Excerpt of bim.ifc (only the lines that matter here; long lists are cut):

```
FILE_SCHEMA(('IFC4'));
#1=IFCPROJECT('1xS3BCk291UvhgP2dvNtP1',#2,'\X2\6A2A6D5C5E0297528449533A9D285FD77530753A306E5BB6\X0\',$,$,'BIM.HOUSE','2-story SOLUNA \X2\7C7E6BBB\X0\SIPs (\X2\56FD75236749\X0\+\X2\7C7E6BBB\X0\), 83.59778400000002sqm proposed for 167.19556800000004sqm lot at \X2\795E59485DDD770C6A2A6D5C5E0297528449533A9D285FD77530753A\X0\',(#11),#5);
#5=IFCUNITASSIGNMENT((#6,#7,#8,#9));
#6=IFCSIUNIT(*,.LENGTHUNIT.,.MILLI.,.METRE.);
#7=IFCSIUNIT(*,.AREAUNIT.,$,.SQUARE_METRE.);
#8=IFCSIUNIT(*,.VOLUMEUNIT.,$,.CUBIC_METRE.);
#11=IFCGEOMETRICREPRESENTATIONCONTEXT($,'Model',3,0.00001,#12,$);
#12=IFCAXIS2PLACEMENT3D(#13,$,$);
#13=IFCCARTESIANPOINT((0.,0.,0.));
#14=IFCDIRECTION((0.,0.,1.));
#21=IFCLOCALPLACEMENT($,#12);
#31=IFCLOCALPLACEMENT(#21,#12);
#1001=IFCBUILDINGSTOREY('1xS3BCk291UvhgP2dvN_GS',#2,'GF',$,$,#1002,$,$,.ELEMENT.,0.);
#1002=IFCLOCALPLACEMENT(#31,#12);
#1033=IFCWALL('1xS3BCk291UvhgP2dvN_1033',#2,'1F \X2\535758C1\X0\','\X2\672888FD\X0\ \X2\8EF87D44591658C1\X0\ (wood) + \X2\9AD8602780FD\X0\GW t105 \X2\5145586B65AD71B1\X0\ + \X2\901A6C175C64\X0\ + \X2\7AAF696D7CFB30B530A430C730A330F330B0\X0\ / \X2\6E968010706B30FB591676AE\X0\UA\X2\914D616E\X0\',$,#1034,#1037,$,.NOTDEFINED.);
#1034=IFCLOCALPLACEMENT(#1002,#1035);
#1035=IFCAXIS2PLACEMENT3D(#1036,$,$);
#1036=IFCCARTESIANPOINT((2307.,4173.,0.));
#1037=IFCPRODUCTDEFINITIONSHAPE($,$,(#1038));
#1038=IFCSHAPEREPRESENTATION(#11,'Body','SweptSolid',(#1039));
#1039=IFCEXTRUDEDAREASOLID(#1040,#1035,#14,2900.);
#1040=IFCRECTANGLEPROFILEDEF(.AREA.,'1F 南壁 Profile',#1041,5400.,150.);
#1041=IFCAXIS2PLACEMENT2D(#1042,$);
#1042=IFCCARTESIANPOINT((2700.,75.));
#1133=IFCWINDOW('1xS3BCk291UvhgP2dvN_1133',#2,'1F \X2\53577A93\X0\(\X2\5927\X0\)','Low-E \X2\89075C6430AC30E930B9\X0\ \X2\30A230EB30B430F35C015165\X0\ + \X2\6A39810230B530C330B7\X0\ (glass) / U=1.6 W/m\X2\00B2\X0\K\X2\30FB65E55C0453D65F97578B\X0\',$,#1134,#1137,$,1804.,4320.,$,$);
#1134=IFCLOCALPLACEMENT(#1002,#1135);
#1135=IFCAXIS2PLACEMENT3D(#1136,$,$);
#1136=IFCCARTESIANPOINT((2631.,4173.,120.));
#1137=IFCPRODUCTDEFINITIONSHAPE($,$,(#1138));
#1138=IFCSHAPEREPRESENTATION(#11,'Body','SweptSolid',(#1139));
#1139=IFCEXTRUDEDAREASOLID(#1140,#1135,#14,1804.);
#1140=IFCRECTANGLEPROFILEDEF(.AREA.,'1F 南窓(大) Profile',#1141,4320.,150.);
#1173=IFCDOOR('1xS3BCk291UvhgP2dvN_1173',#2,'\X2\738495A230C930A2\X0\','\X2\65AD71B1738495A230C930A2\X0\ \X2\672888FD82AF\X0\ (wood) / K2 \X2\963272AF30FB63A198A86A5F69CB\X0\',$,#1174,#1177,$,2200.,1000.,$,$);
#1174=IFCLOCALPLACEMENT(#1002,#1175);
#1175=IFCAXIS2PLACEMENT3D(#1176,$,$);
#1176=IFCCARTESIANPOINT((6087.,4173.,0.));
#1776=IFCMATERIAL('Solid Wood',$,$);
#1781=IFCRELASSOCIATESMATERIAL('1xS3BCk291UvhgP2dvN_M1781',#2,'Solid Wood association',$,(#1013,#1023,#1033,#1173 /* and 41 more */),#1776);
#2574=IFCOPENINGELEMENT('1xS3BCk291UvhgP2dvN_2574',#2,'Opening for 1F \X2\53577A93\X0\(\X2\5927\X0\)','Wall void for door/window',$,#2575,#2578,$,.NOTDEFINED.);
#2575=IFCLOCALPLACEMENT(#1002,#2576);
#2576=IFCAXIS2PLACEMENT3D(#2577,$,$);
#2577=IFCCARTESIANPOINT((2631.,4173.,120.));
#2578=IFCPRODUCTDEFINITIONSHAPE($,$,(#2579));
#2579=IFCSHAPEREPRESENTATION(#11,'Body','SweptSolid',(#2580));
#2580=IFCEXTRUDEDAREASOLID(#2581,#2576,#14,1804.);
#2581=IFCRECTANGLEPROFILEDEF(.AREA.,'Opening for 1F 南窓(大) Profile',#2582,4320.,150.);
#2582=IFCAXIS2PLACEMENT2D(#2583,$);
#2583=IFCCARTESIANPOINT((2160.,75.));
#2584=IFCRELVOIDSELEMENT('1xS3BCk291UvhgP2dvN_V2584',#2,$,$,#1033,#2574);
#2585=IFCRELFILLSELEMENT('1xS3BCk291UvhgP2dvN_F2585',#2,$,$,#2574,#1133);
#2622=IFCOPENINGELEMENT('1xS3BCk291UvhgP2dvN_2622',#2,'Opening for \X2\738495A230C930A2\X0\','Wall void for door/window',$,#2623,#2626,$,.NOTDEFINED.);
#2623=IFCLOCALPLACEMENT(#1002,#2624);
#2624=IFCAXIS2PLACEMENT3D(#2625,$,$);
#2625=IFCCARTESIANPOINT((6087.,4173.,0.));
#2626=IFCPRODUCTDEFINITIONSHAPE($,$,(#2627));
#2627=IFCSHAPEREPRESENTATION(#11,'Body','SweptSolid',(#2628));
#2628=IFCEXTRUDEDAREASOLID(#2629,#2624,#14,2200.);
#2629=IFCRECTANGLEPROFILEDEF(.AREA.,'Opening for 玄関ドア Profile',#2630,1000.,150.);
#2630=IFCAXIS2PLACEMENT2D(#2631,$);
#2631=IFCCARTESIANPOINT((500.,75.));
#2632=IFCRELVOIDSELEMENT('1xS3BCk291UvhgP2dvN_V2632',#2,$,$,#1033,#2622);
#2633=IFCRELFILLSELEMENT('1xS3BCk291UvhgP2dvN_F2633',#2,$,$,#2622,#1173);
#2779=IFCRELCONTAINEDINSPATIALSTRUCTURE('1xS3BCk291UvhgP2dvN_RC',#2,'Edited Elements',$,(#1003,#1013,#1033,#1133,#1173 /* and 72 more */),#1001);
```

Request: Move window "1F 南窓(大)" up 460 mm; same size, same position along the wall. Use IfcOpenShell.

```python
import numpy as np
import ifcopenshell
import ifcopenshell.api.geometry
import ifcopenshell.util.placement
import ifcopenshell.util.unit

model = ifcopenshell.open("bim.ifc")
unit_scale = ifcopenshell.util.unit.calculate_unit_scale(model)

window = model.by_guid("1xS3BCk291UvhgP2dvN_1133")
opening = window.FillsVoids[0].RelatingOpeningElement
dz = 0.46 / unit_scale

shift = np.array([0.0, 0.0, dz])
# The window is not placed relative to its opening, so move both.
for product in (opening, window):
    matrix = ifcopenshell.util.placement.get_local_placement(product.ObjectPlacement)
    matrix[:3, 3] += shift
    ifcopenshell.api.geometry.edit_object_placement(model, product=product, matrix=matrix, is_si=False)

print(f"moved by {dz * unit_scale:+.3f} m")

model.write("bim_rev.ifc")
```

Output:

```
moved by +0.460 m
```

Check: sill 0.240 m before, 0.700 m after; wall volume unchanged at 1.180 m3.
